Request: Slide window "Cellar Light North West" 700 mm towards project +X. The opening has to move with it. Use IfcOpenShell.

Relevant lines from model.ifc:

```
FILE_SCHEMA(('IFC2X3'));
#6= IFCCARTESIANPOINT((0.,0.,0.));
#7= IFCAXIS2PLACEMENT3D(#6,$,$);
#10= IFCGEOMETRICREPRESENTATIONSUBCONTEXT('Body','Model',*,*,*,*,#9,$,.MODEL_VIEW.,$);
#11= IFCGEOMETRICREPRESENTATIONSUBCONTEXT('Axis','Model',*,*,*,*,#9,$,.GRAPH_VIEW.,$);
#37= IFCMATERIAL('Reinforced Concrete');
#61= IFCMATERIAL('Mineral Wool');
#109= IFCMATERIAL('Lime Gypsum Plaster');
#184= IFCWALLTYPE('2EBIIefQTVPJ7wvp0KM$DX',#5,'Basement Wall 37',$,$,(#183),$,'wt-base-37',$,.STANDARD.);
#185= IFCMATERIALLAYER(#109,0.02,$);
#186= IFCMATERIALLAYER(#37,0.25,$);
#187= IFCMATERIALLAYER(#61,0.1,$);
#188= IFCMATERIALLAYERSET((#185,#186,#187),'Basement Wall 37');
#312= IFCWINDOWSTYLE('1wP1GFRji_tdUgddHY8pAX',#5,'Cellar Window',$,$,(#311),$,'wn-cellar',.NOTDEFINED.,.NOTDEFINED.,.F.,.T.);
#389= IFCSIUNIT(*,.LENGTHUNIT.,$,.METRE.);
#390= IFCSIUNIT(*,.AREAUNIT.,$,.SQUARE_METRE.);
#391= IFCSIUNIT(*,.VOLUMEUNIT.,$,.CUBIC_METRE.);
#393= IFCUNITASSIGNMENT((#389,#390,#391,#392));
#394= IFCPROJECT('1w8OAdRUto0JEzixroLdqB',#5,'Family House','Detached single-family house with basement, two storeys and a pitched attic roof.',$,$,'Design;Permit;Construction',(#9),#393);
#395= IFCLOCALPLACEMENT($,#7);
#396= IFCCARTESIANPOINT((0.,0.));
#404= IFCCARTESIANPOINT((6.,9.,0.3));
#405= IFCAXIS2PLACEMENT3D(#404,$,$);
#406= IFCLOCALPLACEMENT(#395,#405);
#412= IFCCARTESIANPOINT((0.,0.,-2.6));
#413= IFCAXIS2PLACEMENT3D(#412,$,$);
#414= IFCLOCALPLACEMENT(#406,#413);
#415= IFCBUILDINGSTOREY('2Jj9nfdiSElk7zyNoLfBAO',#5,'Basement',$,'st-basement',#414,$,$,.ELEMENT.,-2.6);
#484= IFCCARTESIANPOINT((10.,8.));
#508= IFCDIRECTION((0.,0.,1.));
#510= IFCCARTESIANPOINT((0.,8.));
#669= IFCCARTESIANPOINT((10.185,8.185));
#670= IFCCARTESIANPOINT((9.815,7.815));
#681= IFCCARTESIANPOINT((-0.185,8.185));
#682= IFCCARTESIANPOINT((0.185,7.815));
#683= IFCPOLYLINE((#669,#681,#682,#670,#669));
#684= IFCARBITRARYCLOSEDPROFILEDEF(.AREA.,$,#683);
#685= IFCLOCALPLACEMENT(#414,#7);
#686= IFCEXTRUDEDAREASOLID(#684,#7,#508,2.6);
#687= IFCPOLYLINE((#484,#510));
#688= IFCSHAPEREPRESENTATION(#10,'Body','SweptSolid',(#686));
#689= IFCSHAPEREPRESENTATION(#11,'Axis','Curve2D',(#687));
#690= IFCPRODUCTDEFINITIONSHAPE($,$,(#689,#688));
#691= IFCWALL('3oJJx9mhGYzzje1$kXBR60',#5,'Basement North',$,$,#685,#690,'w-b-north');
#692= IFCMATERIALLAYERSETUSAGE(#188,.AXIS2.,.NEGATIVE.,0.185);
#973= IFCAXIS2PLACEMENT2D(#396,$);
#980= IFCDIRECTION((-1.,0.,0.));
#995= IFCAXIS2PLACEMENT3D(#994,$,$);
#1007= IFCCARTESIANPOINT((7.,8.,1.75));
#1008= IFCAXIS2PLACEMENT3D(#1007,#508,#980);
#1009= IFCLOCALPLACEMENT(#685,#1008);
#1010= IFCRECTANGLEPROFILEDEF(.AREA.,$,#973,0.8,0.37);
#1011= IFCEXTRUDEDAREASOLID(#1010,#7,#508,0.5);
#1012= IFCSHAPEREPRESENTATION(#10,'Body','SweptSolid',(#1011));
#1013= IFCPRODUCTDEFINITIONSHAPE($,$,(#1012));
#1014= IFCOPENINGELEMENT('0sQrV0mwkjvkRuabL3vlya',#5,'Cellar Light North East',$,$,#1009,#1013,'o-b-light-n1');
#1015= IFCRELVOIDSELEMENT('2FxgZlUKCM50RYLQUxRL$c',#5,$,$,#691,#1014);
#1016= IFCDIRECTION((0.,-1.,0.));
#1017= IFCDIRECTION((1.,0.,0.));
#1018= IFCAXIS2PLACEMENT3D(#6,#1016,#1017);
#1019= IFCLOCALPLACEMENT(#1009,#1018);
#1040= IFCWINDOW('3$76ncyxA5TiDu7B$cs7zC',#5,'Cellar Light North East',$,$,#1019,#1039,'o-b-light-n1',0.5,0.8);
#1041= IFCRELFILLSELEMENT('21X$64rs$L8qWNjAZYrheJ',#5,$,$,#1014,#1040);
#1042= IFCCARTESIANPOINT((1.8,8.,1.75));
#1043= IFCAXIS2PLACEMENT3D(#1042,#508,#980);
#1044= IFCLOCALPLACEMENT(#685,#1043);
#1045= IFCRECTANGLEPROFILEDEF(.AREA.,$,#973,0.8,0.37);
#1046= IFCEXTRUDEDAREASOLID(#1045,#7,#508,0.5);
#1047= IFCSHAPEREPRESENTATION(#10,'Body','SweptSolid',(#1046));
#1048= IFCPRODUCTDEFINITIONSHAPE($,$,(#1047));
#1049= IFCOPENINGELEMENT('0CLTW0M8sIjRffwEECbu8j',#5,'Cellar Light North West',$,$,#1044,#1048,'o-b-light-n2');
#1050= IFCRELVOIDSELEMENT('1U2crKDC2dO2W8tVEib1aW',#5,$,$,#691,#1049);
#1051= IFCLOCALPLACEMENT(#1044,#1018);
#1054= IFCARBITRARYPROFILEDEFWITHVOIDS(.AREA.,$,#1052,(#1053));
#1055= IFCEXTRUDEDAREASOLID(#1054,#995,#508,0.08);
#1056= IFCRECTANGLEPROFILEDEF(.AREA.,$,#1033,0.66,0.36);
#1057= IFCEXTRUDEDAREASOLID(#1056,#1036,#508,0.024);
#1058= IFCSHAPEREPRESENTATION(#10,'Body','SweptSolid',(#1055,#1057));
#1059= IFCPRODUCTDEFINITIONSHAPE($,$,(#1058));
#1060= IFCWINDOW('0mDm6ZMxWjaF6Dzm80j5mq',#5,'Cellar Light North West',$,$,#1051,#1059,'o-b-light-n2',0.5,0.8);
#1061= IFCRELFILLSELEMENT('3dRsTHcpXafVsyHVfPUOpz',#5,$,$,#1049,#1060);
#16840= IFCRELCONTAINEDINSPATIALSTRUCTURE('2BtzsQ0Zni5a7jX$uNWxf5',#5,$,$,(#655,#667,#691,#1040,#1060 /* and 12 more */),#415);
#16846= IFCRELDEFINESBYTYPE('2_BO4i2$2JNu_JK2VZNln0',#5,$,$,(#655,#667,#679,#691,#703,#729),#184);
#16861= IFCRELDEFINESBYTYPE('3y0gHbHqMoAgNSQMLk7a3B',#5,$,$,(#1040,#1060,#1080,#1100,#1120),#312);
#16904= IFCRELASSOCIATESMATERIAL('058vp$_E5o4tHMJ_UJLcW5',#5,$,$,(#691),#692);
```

```python
import ifcopenshell
import ifcopenshell.api.geometry
import ifcopenshell.util.placement
import ifcopenshell.util.unit

model = ifcopenshell.open("model.ifc")
unit_scale = ifcopenshell.util.unit.calculate_unit_scale(model)

window = model.by_guid("0mDm6ZMxWjaF6Dzm80j5mq")
opening = window.FillsVoids[0].RelatingOpeningElement
wall = opening.VoidsElements[0].RelatingBuildingElement

wall_matrix = ifcopenshell.util.placement.get_local_placement(wall.ObjectPlacement)
shift = wall_matrix[:3, 0] * 0.7 / unit_scale
before = ifcopenshell.util.placement.get_local_placement(window.ObjectPlacement)[:3, 3].copy()

# The window is placed relative to its opening, so it follows when the opening moves.
matrix = ifcopenshell.util.placement.get_local_placement(opening.ObjectPlacement)
matrix[:3, 3] += shift
ifcopenshell.api.geometry.edit_object_placement(
    model, product=opening, matrix=matrix, is_si=False, should_transform_children=True
)

after = ifcopenshell.util.placement.get_local_placement(window.ObjectPlacement)[:3, 3]
print("window moved by", (after - before).round(3) + 0.0)

model.write("model_updated.ifc")
```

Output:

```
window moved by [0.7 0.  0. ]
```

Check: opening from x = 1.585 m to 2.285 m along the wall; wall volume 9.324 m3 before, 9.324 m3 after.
